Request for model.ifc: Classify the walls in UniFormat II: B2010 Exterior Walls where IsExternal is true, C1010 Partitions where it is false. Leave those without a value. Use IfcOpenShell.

First a look at what the model holds.

```python
import ifcopenshell
import ifcopenshell.util.element

model = ifcopenshell.open("model.ifc")
print(model.schema)
print("classifications:", [c.Name for c in model.by_type("IfcClassification")])
values = [ifcopenshell.util.element.get_pset(e, "Pset_WallCommon", "IsExternal") for e in model.by_type("IfcWall")]
for value in (True, False, None):
    print("IsExternal", value, values.count(value))
```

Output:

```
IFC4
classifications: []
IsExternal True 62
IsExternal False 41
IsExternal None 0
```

```python
import ifcopenshell
import ifcopenshell.api.classification
import ifcopenshell.util.element

model = ifcopenshell.open("model.ifc")

system = ifcopenshell.api.classification.add_classification(model, classification="UniFormat II")

walls = model.by_type("IfcWall")
external = {e: ifcopenshell.util.element.get_pset(e, "Pset_WallCommon", "IsExternal") for e in walls}
for flag, code, name in ((True, "B2010", "Exterior Walls"), (False, "C1010", "Partitions")):
    products = [e for e in walls if external[e] is flag]
    ifcopenshell.api.classification.add_reference(
        model, products=products, classification=system, identification=code, name=name
    )
    print(code, len(products))

model.write("model_v2.ifc")
```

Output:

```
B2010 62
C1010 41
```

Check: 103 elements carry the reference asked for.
